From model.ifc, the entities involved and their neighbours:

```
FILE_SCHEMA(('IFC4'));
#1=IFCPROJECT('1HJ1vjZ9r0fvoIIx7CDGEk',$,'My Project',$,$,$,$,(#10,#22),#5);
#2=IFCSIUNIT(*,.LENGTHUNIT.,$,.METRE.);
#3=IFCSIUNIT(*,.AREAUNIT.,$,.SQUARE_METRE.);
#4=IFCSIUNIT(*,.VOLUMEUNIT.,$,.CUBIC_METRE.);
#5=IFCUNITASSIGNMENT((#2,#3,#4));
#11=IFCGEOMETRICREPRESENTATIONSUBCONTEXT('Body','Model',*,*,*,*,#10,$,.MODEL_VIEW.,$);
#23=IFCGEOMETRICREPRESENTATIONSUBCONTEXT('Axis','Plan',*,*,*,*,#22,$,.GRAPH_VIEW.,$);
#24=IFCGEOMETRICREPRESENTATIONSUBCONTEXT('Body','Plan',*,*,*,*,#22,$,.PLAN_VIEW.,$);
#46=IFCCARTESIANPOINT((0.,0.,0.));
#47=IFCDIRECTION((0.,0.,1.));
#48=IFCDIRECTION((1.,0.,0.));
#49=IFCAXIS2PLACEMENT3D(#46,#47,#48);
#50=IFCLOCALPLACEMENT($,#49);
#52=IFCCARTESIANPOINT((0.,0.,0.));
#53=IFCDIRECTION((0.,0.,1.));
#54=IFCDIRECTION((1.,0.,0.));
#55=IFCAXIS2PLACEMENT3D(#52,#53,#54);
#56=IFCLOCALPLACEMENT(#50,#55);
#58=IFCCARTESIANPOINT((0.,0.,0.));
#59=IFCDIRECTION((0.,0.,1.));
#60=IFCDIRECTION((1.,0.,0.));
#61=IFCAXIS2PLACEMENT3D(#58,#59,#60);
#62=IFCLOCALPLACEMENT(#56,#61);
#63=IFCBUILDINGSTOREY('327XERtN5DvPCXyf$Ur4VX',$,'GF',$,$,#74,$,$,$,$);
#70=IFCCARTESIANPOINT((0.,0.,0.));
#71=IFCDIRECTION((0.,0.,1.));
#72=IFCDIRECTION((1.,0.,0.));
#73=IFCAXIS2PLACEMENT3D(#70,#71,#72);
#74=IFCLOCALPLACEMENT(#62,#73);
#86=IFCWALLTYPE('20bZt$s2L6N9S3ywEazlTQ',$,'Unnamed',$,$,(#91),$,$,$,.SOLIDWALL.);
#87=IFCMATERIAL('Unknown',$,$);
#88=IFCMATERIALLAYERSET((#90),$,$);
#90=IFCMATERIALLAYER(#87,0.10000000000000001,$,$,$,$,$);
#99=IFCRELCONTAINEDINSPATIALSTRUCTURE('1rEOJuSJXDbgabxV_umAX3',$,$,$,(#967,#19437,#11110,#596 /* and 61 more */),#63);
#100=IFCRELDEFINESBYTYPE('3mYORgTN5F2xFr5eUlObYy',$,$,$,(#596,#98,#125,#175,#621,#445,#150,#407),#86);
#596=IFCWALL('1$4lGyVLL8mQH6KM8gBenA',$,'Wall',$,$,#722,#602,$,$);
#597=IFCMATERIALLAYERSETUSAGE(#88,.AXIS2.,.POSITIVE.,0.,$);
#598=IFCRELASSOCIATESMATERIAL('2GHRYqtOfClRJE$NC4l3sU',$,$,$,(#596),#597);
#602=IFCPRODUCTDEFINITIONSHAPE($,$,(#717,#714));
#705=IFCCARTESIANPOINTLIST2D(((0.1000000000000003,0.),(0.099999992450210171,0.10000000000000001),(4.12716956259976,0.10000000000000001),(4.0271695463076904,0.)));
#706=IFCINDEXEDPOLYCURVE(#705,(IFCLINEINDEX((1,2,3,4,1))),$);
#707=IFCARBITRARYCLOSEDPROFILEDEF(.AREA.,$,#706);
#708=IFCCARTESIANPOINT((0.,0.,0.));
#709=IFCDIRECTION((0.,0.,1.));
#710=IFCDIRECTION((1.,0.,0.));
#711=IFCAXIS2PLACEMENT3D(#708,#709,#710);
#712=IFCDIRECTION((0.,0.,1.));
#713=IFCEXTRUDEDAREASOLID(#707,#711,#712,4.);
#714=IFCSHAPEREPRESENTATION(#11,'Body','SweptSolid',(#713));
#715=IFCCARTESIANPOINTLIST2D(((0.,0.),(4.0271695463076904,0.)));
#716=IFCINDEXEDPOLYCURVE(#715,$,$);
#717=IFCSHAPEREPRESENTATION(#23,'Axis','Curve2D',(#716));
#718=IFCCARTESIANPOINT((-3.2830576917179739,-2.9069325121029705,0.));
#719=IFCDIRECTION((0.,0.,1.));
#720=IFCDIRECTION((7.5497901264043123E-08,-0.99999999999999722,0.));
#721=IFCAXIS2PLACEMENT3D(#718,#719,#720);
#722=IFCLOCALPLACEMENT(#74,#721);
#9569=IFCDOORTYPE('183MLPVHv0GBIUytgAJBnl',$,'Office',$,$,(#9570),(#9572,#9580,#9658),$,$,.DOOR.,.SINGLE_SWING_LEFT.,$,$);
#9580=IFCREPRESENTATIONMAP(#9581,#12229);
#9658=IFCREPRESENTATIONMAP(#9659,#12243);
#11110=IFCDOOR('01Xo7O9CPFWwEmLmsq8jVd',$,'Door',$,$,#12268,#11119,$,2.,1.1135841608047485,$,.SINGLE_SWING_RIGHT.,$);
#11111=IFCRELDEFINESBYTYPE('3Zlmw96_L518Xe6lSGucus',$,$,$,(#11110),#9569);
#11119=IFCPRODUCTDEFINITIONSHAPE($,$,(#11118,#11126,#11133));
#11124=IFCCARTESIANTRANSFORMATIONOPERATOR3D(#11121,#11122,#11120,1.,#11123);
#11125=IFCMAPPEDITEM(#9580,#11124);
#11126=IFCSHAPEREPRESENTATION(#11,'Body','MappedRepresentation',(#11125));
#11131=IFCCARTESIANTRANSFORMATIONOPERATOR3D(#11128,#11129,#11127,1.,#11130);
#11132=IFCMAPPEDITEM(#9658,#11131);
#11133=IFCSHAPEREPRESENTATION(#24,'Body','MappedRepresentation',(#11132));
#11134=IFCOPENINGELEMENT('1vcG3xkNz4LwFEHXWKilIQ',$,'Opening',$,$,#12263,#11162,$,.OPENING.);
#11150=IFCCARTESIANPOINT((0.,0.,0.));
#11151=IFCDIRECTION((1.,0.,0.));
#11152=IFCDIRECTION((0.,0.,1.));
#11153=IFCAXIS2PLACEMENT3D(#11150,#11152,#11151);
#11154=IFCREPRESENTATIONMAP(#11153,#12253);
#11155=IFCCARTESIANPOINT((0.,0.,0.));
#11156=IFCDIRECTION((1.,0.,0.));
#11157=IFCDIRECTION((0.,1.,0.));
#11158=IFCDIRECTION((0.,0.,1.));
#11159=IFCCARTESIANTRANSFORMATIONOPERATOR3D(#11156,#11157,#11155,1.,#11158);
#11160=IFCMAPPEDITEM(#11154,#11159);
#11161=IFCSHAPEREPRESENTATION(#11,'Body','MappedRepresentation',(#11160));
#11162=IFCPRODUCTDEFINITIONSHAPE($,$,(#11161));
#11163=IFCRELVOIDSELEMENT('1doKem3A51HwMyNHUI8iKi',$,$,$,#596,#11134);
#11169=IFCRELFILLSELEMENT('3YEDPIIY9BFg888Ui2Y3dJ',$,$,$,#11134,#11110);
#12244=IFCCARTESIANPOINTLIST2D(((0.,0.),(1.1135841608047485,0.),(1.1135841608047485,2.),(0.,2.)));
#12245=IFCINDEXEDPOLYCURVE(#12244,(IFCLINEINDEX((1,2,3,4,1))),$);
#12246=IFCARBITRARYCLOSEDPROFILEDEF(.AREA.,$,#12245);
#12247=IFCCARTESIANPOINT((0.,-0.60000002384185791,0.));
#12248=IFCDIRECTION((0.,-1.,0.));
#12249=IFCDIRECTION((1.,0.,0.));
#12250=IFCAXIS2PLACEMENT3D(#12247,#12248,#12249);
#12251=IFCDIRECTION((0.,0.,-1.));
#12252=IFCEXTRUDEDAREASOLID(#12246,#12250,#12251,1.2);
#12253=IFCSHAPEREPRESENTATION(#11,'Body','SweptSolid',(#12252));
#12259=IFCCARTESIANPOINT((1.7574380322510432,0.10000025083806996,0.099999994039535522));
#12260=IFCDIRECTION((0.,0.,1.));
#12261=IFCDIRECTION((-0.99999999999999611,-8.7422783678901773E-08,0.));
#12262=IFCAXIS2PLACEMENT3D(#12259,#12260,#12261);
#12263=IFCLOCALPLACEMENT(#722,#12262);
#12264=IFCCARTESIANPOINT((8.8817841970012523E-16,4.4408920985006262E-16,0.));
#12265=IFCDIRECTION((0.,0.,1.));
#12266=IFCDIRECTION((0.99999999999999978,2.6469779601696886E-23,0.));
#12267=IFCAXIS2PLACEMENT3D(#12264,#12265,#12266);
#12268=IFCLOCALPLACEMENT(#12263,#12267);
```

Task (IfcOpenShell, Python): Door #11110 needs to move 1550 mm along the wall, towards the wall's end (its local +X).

```python
import ifcopenshell
import ifcopenshell.api.geometry
import ifcopenshell.util.placement

model = ifcopenshell.open("model.ifc")

door = model.by_guid("01Xo7O9CPFWwEmLmsq8jVd")
opening = door.FillsVoids[0].RelatingOpeningElement
wall = opening.VoidsElements[0].RelatingBuildingElement

wall_matrix = ifcopenshell.util.placement.get_local_placement(wall.ObjectPlacement)
shift = wall_matrix[:3, 0] * 1.55
before = ifcopenshell.util.placement.get_local_placement(door.ObjectPlacement)[:3, 3].copy()

# The door is placed relative to its opening, so it follows when the opening moves.
matrix = ifcopenshell.util.placement.get_local_placement(opening.ObjectPlacement)
matrix[:3, 3] += shift
ifcopenshell.api.geometry.edit_object_placement(
    model, product=opening, matrix=matrix, is_si=False, should_transform_children=True
)

after = ifcopenshell.util.placement.get_local_placement(door.ObjectPlacement)[:3, 3]
print("door moved by", (after - before).round(3) + 0.0)

model.write("model_edited.ifc")
```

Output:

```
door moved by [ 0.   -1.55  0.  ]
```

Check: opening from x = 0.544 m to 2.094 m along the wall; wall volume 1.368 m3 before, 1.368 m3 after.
